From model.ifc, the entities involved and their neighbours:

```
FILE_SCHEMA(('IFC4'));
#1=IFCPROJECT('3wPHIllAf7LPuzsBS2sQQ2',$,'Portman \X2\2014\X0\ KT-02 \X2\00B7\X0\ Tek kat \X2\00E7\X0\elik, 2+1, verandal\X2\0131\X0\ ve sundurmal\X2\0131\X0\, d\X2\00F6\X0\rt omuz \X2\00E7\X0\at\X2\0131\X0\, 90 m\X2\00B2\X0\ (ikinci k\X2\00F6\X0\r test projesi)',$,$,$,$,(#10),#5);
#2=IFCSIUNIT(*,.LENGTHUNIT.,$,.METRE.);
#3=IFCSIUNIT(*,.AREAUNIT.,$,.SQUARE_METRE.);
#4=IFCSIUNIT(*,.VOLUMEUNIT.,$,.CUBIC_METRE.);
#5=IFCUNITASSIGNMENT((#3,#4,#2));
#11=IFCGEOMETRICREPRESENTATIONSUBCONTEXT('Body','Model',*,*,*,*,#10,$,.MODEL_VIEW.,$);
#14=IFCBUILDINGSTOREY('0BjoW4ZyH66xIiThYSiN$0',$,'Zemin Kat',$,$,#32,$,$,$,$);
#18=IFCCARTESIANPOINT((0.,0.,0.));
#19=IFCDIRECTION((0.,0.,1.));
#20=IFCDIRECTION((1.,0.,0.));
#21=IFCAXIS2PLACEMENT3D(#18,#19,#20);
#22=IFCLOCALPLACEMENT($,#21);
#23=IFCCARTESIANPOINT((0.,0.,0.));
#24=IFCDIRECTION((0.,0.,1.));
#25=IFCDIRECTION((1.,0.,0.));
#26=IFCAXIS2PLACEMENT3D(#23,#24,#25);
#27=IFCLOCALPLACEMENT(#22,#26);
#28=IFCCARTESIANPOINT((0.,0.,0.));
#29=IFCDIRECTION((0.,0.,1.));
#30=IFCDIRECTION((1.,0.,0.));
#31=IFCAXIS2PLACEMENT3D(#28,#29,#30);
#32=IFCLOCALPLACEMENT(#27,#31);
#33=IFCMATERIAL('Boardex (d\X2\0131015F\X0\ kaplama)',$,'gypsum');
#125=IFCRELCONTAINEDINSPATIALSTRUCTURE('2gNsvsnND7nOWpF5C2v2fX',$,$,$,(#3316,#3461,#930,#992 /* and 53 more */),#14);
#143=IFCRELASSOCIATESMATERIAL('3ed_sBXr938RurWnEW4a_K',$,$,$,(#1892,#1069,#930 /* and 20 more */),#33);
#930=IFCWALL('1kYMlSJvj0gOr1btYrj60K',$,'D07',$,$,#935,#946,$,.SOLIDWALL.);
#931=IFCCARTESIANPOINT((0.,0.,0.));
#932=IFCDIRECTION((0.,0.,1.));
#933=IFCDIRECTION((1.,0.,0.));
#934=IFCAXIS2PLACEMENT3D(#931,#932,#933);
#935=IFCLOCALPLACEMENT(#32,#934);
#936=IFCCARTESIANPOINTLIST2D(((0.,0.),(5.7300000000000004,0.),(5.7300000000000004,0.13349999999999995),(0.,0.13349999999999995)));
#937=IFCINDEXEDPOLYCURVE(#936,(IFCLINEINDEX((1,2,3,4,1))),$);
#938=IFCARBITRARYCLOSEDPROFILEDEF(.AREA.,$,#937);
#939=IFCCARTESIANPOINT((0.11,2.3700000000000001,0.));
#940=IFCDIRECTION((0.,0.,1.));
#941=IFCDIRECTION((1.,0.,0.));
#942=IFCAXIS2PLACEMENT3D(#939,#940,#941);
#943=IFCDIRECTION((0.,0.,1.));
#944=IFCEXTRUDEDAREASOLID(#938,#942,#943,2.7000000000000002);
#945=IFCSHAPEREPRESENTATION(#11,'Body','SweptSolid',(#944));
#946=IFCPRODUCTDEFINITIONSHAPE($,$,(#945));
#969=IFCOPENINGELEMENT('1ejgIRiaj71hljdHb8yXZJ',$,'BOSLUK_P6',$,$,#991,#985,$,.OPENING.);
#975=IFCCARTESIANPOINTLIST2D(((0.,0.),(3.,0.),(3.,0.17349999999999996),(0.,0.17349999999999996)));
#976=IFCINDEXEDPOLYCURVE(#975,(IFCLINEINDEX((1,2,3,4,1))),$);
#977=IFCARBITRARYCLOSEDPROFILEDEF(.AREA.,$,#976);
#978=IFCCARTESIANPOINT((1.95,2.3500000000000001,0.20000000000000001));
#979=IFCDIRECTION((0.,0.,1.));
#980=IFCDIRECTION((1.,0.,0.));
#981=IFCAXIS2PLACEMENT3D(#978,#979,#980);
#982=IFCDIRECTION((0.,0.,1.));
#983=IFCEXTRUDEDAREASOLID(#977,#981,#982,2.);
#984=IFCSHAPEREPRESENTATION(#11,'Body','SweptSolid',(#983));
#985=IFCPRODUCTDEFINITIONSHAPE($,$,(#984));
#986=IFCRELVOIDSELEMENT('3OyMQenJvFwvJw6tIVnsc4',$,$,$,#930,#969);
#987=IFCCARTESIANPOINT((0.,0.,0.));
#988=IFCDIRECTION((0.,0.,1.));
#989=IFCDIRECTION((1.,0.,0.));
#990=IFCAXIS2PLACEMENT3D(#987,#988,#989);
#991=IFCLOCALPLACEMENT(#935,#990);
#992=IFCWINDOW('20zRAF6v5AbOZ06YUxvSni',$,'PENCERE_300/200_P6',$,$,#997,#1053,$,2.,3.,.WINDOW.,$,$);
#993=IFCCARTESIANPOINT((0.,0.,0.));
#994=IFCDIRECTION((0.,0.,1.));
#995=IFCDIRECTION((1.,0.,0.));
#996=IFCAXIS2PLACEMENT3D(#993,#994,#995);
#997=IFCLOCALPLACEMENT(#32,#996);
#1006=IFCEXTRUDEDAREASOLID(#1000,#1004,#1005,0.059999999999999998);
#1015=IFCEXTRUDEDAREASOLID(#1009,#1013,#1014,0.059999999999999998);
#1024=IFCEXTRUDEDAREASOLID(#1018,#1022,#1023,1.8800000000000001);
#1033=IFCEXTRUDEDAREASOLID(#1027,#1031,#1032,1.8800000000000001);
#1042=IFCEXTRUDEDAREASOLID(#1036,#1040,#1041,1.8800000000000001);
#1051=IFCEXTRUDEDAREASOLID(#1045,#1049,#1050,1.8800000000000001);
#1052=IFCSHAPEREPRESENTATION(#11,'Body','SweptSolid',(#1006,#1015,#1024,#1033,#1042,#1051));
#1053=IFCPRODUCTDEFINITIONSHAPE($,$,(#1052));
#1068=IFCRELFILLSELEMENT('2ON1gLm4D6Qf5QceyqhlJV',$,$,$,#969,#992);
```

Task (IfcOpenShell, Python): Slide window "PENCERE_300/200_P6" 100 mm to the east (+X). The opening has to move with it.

```python
import ifcopenshell
import ifcopenshell.api.geometry
import ifcopenshell.util.placement

model = ifcopenshell.open("model.ifc")

window = model.by_guid("20zRAF6v5AbOZ06YUxvSni")
opening = window.FillsVoids[0].RelatingOpeningElement
wall = opening.VoidsElements[0].RelatingBuildingElement

wall_matrix = ifcopenshell.util.placement.get_local_placement(wall.ObjectPlacement)
shift = wall_matrix[:3, 0] * 0.1
before = ifcopenshell.util.placement.get_local_placement(window.ObjectPlacement)[:3, 3].copy()

# The window is not placed relative to its opening, so move both.
for product in (opening, window):
    matrix = ifcopenshell.util.placement.get_local_placement(product.ObjectPlacement)
    matrix[:3, 3] += shift
    ifcopenshell.api.geometry.edit_object_placement(model, product=product, matrix=matrix, is_si=False)

after = ifcopenshell.util.placement.get_local_placement(window.ObjectPlacement)[:3, 3]
print("window moved by", (after - before).round(3) + 0.0)

model.write("model-out.ifc")
```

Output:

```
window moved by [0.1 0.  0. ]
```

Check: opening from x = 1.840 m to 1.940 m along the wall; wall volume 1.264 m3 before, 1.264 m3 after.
